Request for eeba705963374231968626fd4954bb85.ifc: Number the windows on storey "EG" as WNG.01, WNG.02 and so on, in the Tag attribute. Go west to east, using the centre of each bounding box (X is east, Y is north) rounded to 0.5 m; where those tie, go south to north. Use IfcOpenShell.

First a look at what the model holds.

```python
import ifcopenshell
import ifcopenshell.util.element
import ifcopenshell.util.placement

model = ifcopenshell.open("eeba705963374231968626fd4954bb85.ifc")
print(model.schema)
storey = next(s for s in model.by_type("IfcBuildingStorey") if s.Name == "EG")
windows = [e for e in ifcopenshell.util.element.get_decomposition(storey) if e.is_a("IfcWindow")]
for e in sorted(windows, key=lambda e: e.id()):
    origin = ifcopenshell.util.placement.get_local_placement(e.ObjectPlacement)[:3, 3]
    print(e.id(), e.Tag, e.Name, origin.round(2) + 0.0, sep=" | ")
```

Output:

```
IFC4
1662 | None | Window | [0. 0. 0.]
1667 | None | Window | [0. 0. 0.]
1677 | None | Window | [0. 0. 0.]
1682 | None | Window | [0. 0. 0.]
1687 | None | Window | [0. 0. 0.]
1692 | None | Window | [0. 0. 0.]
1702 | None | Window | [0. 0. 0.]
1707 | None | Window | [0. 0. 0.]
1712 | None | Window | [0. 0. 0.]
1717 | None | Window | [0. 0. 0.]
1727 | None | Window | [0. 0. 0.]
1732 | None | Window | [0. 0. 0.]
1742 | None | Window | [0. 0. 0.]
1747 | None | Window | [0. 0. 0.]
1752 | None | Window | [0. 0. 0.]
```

```python
import ifcopenshell
import ifcopenshell.geom
import ifcopenshell.util.element
import ifcopenshell.util.shape

model = ifcopenshell.open("eeba705963374231968626fd4954bb85.ifc")
settings = ifcopenshell.geom.settings()
settings.set("use-world-coords", True)


def centre(element):
    shape = ifcopenshell.geom.create_shape(settings, element)
    return ifcopenshell.util.shape.get_bbox_centroid(shape.geometry)


storey = next(s for s in model.by_type("IfcBuildingStorey") if s.Name == "EG")
windows = [e for e in ifcopenshell.util.element.get_decomposition(storey) if e.is_a("IfcWindow")]

# Insertion points can sit at a corner or the storey origin, so sort by the geometry (in metres).
centres = {e: centre(e) for e in windows}
windows.sort(key=lambda e: (round(centres[e][0] / 0.5), centres[e][1]))

for i, e in enumerate(windows, start=1):
    number = f"WNG.{i:02d}"
    e.Tag = number
    print(e.id(), number)

model.write("eeba705963374231968626fd4954bb85-out.ifc")
```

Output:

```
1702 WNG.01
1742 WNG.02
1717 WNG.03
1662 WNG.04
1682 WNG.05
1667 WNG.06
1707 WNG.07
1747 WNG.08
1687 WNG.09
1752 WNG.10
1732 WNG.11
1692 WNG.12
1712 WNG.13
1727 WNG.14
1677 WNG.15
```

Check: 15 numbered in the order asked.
